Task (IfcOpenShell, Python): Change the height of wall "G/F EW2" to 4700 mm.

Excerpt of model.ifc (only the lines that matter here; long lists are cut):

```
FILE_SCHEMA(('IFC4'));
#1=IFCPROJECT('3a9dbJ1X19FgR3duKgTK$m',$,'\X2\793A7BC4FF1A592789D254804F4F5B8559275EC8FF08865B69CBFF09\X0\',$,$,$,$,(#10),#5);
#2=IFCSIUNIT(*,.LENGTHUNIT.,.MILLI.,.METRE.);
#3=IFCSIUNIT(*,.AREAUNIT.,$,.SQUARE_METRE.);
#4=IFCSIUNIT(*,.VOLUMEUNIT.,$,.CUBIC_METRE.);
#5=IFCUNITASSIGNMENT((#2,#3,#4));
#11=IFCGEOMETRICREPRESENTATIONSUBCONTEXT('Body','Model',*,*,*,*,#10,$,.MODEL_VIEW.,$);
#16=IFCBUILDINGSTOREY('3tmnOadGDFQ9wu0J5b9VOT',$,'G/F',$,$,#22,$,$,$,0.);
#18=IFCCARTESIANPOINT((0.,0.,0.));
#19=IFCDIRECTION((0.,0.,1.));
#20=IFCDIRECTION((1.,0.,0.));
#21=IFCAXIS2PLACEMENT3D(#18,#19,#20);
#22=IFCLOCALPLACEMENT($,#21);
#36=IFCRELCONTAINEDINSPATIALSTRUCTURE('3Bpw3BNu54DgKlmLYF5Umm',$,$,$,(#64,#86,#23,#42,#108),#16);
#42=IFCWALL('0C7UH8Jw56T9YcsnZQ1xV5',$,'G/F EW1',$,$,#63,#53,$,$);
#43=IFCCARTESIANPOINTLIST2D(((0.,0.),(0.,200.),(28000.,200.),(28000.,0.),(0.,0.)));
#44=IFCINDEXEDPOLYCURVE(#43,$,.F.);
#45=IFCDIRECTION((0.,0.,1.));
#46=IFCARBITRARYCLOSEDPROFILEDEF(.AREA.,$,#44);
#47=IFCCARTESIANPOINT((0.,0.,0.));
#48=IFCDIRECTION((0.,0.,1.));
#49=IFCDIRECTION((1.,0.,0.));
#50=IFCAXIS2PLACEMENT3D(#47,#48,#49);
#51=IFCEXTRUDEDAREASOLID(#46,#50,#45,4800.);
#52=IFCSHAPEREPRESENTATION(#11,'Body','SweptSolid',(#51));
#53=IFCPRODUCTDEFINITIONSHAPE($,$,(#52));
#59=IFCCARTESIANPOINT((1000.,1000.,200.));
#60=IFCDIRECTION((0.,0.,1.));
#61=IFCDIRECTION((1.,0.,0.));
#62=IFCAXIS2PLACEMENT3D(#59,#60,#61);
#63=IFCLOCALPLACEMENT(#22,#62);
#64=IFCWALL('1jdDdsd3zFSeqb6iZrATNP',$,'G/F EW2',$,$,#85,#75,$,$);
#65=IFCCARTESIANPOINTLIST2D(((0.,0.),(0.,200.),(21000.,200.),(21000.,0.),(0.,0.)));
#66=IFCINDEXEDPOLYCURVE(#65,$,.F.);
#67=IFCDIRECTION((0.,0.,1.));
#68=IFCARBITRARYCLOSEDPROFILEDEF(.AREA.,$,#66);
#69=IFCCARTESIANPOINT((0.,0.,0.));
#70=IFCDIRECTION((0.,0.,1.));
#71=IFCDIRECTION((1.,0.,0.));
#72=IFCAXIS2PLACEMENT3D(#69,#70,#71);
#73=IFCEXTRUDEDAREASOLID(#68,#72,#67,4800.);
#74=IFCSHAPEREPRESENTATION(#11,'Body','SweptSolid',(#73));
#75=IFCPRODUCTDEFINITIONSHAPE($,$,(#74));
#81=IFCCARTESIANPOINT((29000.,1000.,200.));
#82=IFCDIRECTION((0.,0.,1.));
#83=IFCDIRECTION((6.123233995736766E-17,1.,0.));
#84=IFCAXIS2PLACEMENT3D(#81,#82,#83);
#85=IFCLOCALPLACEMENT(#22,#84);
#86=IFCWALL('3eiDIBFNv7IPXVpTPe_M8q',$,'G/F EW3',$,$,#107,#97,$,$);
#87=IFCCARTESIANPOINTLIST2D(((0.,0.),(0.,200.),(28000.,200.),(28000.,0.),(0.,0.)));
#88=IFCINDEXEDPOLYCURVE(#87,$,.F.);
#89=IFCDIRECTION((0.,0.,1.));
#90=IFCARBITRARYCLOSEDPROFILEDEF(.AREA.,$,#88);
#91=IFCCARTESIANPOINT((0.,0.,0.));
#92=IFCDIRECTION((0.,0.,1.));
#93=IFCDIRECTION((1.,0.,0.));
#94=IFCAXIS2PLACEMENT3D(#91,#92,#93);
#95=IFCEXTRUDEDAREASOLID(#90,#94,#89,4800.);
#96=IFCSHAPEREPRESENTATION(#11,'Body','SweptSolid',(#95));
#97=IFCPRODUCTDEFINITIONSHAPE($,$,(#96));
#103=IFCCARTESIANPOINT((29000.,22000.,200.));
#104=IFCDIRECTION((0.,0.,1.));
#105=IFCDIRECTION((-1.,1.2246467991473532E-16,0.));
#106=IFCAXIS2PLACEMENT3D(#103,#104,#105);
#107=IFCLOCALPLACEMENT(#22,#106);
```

```python
import ifcopenshell
import ifcopenshell.geom
import ifcopenshell.util.representation
import ifcopenshell.util.shape

model = ifcopenshell.open("model.ifc")
settings = ifcopenshell.geom.settings()


def volume(element):
    """Net volume in cubic metres, openings subtracted."""
    shape = ifcopenshell.geom.create_shape(settings, element)
    return ifcopenshell.util.shape.get_volume(shape.geometry)


wall = model.by_guid("1jdDdsd3zFSeqb6iZrATNP")
before = volume(wall)

body = ifcopenshell.util.representation.get_representation(wall, "Model", "Body")
solid = body.Items[0]
old_height = solid.Depth
solid.Depth = 4700.0
after = volume(wall)

print(f"height {old_height:g} -> {solid.Depth:g}, volume {before:.3f} -> {after:.3f} m3")

model.write("model_updated.ifc")
```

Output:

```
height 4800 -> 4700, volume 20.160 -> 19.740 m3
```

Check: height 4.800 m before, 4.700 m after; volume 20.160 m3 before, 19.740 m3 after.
